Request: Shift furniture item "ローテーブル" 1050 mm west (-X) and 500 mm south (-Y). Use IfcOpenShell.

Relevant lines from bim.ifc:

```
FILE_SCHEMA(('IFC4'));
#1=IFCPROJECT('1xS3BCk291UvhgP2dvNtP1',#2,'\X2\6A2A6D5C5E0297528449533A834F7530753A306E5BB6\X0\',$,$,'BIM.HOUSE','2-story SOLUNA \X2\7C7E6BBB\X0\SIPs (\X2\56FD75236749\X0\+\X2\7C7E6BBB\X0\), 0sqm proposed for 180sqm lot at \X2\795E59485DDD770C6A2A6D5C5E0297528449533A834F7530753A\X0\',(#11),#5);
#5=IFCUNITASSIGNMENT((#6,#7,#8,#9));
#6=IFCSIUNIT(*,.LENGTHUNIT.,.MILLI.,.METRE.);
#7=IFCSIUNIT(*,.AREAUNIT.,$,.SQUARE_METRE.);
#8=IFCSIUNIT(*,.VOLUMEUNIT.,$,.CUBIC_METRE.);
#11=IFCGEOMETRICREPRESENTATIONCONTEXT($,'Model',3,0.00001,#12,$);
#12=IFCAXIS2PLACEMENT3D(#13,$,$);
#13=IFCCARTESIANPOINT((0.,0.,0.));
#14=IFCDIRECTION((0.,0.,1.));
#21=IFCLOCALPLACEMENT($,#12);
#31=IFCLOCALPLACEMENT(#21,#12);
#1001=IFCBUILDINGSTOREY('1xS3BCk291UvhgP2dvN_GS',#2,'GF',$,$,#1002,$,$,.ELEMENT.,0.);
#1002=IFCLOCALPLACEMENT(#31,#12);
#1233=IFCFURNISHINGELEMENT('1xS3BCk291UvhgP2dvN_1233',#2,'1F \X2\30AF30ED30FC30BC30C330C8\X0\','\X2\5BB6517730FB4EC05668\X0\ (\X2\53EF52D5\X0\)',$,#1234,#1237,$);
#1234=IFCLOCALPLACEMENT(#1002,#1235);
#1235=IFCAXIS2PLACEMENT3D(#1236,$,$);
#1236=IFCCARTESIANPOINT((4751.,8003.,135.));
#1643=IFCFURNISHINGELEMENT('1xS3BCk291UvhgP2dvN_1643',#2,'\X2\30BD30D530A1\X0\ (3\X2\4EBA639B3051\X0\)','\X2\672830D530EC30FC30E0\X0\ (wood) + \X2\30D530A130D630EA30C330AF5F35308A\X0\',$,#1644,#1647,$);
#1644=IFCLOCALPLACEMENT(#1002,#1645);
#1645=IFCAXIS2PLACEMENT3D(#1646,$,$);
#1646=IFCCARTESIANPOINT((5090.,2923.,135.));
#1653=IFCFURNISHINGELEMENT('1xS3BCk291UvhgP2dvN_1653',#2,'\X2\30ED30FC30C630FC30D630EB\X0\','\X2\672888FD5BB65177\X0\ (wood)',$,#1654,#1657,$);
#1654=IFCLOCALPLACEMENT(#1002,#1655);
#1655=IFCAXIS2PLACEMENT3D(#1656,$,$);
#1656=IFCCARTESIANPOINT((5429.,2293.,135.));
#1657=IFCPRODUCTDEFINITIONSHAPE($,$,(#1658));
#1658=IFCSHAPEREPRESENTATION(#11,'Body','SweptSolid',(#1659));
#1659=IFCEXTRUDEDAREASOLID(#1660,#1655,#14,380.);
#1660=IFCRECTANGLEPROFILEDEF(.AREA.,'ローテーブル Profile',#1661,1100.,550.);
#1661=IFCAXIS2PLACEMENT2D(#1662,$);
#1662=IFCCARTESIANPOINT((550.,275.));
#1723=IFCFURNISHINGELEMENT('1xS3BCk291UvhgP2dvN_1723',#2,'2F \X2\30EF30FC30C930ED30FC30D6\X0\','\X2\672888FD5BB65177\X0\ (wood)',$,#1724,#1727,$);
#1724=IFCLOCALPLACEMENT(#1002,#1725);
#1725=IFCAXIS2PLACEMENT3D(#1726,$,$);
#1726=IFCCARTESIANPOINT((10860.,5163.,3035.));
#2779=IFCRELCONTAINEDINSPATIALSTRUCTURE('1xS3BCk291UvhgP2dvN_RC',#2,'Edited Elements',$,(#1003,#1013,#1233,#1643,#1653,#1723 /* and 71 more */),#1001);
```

```python
import ifcopenshell
import ifcopenshell.api.geometry
import ifcopenshell.util.placement
import ifcopenshell.util.unit

model = ifcopenshell.open("bim.ifc")
unit_scale = ifcopenshell.util.unit.calculate_unit_scale(model)

item = model.by_id(1653)
matrix = ifcopenshell.util.placement.get_local_placement(item.ObjectPlacement)
matrix[0, 3] -= 1.05 / unit_scale
matrix[1, 3] -= 0.5 / unit_scale
ifcopenshell.api.geometry.edit_object_placement(model, product=item, matrix=matrix, is_si=False)

print(ifcopenshell.util.placement.get_local_placement(item.ObjectPlacement).round(3) + 0.0)

model.write("bim-out.ifc")
```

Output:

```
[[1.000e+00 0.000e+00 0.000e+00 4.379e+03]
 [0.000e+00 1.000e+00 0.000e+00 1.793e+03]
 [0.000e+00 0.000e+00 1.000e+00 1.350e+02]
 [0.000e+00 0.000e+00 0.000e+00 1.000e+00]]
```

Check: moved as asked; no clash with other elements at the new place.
